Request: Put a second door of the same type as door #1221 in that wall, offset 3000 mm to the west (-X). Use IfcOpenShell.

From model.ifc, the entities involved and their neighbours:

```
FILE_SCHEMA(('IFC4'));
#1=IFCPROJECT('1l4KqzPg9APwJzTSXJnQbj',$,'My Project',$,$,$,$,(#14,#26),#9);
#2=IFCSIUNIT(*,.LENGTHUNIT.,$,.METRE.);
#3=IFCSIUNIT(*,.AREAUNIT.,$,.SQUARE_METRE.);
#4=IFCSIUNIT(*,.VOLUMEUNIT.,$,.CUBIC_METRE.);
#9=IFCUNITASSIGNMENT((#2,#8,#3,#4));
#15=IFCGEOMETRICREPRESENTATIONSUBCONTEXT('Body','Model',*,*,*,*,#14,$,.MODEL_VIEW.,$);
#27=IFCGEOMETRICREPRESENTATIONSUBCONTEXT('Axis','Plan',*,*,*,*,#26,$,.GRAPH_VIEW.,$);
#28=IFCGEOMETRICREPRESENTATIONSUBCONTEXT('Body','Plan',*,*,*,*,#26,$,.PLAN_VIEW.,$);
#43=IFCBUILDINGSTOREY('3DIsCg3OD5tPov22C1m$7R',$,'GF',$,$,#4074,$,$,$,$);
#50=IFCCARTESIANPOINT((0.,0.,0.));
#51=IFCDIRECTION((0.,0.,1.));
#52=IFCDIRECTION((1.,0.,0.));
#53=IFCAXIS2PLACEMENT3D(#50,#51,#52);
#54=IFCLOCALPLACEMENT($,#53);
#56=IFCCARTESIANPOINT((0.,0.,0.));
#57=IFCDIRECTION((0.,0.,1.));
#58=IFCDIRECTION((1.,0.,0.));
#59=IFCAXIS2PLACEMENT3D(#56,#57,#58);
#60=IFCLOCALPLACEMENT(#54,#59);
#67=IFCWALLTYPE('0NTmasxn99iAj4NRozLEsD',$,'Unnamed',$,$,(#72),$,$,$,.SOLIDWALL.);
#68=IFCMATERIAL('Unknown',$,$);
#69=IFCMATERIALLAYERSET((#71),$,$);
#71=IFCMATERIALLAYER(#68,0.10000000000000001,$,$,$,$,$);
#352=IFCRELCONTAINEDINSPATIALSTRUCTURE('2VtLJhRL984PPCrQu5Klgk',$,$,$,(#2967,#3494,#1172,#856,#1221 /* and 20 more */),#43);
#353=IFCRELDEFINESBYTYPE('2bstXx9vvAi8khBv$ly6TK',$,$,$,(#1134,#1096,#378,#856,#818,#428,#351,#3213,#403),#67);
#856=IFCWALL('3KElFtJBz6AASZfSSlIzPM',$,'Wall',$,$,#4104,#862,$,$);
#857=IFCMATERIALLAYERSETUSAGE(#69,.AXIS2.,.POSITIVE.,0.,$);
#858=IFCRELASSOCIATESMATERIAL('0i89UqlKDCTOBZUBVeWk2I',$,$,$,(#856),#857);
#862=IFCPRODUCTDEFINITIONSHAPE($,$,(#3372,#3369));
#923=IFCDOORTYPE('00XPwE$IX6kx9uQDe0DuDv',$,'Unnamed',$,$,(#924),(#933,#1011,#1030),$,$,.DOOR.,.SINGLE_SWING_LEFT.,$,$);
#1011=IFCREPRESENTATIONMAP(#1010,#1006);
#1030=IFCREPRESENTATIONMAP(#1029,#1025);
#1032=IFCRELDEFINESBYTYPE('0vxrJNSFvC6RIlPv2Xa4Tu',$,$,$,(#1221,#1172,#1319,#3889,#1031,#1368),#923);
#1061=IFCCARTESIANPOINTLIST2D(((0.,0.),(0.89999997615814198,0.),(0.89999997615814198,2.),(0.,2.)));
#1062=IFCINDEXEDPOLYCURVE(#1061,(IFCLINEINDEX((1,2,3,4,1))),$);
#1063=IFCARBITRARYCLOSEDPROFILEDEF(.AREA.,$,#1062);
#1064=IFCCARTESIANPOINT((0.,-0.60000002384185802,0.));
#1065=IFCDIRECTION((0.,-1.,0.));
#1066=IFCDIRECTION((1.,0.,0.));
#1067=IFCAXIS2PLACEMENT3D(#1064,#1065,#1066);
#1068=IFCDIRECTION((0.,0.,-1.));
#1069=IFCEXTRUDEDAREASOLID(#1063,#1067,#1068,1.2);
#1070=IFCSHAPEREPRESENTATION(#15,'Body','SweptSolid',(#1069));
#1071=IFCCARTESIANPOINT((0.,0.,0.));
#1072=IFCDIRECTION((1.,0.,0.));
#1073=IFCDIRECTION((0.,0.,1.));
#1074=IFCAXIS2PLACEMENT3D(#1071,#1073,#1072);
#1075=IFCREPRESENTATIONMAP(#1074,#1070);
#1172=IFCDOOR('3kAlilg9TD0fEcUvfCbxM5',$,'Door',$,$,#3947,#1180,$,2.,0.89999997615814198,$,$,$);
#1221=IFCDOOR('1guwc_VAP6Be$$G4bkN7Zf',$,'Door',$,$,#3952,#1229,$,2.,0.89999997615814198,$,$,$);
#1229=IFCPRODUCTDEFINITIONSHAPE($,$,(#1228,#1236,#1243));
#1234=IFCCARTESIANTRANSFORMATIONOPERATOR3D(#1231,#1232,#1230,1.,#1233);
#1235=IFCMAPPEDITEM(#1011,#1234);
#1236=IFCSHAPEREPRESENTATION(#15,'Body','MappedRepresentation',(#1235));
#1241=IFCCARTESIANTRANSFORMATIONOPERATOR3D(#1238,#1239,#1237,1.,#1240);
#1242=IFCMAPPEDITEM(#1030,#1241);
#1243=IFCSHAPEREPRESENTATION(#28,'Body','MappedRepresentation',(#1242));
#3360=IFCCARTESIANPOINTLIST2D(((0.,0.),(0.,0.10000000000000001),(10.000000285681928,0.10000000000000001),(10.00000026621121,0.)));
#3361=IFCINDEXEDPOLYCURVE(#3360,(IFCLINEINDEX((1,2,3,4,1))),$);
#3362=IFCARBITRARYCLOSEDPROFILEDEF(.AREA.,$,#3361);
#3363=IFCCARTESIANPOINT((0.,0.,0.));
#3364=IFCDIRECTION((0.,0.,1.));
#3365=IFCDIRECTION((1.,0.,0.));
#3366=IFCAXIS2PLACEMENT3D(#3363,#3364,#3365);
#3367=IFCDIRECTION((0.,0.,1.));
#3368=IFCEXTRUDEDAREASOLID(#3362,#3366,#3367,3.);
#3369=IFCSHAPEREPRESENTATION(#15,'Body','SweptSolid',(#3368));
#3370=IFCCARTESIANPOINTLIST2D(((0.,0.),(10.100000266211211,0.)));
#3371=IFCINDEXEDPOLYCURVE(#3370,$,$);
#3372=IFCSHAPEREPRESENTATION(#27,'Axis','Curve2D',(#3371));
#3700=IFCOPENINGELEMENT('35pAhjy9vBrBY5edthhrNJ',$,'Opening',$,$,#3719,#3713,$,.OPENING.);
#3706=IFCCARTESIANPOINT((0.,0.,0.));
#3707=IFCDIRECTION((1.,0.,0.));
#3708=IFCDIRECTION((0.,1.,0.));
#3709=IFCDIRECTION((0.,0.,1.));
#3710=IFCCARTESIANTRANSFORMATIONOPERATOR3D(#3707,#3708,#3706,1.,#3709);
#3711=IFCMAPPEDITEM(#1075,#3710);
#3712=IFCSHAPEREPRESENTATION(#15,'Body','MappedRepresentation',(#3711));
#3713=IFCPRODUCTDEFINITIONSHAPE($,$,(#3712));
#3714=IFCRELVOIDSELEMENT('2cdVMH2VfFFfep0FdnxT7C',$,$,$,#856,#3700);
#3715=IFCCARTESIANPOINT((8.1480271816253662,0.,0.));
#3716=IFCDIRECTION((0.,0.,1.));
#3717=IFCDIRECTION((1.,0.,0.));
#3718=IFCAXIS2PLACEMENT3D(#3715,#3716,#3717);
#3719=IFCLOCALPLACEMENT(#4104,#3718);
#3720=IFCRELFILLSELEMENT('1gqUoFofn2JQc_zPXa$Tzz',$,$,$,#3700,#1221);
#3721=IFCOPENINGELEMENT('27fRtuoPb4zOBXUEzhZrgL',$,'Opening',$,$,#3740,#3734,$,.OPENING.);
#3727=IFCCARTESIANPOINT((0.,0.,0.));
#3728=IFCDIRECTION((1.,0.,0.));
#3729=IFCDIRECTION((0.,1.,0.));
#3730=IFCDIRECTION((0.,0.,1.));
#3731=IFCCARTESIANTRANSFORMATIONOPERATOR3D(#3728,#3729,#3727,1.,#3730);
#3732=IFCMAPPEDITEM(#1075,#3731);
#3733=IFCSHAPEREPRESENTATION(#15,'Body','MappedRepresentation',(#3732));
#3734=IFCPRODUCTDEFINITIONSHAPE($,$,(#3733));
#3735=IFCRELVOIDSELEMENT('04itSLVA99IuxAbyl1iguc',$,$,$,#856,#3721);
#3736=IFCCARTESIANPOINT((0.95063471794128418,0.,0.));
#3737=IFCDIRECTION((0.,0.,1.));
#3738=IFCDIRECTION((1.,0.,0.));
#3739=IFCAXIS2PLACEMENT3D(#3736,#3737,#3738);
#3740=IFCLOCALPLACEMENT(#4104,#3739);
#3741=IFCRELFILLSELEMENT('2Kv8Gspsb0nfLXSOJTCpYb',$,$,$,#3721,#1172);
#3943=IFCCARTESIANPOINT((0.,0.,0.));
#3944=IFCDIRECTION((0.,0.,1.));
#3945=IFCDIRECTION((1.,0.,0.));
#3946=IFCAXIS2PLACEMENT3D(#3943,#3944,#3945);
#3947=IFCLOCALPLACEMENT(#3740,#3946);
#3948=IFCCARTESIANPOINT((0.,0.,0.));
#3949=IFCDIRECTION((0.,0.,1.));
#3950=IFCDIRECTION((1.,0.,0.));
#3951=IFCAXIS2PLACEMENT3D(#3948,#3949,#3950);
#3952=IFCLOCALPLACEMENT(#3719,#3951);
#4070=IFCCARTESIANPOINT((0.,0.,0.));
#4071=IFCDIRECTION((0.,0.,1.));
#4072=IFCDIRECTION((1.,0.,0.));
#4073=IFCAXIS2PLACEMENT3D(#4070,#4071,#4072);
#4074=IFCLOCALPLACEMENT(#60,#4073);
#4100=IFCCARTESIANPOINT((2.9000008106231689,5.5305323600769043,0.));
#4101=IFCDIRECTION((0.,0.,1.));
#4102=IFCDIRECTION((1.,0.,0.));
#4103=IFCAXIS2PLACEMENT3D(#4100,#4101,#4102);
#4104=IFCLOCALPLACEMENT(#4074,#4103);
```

```python
import ifcopenshell
import ifcopenshell.api.feature
import ifcopenshell.api.geometry
import ifcopenshell.api.root
import ifcopenshell.geom
import ifcopenshell.util.element
import ifcopenshell.util.placement
import ifcopenshell.util.shape
import ifcopenshell.util.unit

model = ifcopenshell.open("model.ifc")
unit_scale = ifcopenshell.util.unit.calculate_unit_scale(model)
settings = ifcopenshell.geom.settings()


def volume(element):
    """Net volume in cubic metres, openings subtracted."""
    shape = ifcopenshell.geom.create_shape(settings, element)
    return ifcopenshell.util.shape.get_volume(shape.geometry)


door = model.by_guid("1guwc_VAP6Be$$G4bkN7Zf")
opening = door.FillsVoids[0].RelatingOpeningElement
wall = opening.VoidsElements[0].RelatingBuildingElement
before = volume(wall)
shift = ifcopenshell.util.placement.get_local_placement(wall.ObjectPlacement)[:3, 0] * -3 / unit_scale

# copy_class copies the void relationship, type, container and properties, but no geometry.
new_opening = ifcopenshell.api.root.copy_class(model, product=opening)
new_opening.Representation = ifcopenshell.util.element.copy_deep(
    model, opening.Representation, exclude=["IfcGeometricRepresentationContext", "IfcRepresentationMap"]
)
new_door = ifcopenshell.api.root.copy_class(model, product=door)
new_door.Representation = ifcopenshell.util.element.copy_deep(
    model, door.Representation, exclude=["IfcGeometricRepresentationContext", "IfcRepresentationMap"]
)
ifcopenshell.api.feature.add_filling(model, opening=new_opening, element=new_door)

for old, new in ((opening, new_opening), (door, new_door)):
    matrix = ifcopenshell.util.placement.get_local_placement(old.ObjectPlacement)
    matrix[:3, 3] += shift
    ifcopenshell.api.geometry.edit_object_placement(model, product=new, matrix=matrix, is_si=False)

after = volume(wall)

print(f"wall volume {before:.3f} -> {after:.3f} m3")

model.write("model_edited.ifc")
```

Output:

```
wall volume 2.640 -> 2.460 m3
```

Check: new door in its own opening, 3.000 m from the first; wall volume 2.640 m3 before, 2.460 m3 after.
